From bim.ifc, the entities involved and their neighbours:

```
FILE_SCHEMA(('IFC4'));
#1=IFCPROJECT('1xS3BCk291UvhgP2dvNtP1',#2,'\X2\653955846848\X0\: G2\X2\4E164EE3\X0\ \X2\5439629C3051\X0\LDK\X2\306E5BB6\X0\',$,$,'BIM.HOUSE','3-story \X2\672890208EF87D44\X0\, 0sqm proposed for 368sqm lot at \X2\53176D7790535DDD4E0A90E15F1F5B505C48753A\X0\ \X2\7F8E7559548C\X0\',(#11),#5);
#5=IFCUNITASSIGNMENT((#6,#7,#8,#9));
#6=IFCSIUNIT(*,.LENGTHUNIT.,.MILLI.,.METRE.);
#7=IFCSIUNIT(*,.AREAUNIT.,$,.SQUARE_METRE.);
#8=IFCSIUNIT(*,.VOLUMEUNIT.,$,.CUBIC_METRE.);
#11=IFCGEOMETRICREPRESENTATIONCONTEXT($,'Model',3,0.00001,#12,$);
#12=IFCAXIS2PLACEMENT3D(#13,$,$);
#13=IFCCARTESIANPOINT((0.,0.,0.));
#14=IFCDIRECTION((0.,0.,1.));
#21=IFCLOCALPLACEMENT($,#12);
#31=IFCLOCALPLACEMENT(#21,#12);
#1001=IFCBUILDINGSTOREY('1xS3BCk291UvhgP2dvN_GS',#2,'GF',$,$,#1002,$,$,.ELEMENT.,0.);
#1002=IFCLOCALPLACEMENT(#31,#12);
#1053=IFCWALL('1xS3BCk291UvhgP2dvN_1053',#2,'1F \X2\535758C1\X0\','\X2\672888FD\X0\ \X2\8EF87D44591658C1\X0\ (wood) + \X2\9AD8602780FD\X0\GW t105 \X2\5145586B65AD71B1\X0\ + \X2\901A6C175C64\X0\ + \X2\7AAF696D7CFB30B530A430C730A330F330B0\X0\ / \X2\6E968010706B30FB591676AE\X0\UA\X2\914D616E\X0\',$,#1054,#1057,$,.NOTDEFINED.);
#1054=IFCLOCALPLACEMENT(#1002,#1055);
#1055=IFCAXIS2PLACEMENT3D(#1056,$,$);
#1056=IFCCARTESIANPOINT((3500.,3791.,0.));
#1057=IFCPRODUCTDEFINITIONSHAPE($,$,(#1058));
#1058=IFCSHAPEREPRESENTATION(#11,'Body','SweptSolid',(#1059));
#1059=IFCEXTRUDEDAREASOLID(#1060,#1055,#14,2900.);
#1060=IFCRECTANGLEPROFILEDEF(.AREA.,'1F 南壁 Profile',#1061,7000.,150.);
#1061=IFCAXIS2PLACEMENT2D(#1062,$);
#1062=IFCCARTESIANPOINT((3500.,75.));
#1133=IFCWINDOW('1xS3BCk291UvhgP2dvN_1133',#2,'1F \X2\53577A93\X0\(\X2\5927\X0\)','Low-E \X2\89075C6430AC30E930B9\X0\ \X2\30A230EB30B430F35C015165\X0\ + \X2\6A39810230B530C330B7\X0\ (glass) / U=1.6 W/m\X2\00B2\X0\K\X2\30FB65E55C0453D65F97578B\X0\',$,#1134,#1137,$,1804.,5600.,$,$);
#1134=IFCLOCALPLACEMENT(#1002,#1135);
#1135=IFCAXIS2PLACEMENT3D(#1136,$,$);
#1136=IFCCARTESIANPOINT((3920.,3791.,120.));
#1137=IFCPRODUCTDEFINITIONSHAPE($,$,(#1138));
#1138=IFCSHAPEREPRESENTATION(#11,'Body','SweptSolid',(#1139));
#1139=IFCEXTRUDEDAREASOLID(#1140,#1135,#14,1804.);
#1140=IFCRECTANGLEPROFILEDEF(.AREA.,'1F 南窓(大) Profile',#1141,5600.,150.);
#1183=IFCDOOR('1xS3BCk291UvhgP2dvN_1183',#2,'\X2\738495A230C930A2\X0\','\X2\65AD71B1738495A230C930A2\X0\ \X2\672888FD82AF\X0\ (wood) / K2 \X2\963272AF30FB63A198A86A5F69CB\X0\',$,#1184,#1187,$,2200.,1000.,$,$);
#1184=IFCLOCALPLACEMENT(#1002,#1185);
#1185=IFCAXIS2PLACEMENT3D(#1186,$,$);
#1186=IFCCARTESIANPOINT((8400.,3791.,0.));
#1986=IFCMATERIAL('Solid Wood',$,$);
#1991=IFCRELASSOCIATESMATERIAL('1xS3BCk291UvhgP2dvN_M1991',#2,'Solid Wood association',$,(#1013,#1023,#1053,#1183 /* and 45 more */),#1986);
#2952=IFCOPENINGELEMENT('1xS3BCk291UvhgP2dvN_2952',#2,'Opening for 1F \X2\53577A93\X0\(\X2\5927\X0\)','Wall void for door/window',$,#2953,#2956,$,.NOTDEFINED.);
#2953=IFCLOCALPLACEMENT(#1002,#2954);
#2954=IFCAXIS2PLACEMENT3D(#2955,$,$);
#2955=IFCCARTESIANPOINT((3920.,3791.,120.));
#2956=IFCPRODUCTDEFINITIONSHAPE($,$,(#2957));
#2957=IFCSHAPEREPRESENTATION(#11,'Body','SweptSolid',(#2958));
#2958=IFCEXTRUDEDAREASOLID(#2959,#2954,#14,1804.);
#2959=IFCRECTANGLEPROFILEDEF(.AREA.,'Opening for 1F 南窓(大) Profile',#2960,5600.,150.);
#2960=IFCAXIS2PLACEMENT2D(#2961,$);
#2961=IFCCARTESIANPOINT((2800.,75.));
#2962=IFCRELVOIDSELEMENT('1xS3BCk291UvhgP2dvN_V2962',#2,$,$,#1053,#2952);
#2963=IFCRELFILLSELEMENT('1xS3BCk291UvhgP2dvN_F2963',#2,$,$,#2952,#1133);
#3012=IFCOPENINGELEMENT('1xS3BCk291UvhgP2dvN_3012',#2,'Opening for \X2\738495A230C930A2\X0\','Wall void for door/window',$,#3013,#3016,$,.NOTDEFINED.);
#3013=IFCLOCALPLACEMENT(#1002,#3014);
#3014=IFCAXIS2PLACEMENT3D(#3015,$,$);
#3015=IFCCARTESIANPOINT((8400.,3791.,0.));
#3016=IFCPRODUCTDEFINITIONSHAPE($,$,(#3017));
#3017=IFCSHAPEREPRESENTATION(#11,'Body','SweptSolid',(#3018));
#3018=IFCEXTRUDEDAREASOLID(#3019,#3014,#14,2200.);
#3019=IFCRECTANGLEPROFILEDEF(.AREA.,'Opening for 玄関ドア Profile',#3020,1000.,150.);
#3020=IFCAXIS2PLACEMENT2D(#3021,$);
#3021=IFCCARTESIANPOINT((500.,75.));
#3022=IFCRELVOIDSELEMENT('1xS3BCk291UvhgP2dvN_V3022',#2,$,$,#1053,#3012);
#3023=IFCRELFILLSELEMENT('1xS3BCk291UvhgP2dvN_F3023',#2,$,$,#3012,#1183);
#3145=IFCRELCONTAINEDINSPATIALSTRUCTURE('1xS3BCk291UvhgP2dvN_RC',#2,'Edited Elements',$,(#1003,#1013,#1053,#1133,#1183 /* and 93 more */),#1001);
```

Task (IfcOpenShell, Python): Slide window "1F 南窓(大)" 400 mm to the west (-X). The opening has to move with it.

```python
import ifcopenshell
import ifcopenshell.api.geometry
import ifcopenshell.util.placement

model = ifcopenshell.open("bim.ifc")

window = model.by_id(1133)
opening = window.FillsVoids[0].RelatingOpeningElement
wall = opening.VoidsElements[0].RelatingBuildingElement

wall_matrix = ifcopenshell.util.placement.get_local_placement(wall.ObjectPlacement)
shift = wall_matrix[:3, 0] * -400.0
before = ifcopenshell.util.placement.get_local_placement(window.ObjectPlacement)[:3, 3].copy()

# The window is not placed relative to its opening, so move both.
for product in (opening, window):
    matrix = ifcopenshell.util.placement.get_local_placement(product.ObjectPlacement)
    matrix[:3, 3] += shift
    ifcopenshell.api.geometry.edit_object_placement(model, product=product, matrix=matrix, is_si=False)

after = ifcopenshell.util.placement.get_local_placement(window.ObjectPlacement)[:3, 3]
print("window moved by", (after - before).round(3) + 0.0)

model.write("bim_rev.ifc")
```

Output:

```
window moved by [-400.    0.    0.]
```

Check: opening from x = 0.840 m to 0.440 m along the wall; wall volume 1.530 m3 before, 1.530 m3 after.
